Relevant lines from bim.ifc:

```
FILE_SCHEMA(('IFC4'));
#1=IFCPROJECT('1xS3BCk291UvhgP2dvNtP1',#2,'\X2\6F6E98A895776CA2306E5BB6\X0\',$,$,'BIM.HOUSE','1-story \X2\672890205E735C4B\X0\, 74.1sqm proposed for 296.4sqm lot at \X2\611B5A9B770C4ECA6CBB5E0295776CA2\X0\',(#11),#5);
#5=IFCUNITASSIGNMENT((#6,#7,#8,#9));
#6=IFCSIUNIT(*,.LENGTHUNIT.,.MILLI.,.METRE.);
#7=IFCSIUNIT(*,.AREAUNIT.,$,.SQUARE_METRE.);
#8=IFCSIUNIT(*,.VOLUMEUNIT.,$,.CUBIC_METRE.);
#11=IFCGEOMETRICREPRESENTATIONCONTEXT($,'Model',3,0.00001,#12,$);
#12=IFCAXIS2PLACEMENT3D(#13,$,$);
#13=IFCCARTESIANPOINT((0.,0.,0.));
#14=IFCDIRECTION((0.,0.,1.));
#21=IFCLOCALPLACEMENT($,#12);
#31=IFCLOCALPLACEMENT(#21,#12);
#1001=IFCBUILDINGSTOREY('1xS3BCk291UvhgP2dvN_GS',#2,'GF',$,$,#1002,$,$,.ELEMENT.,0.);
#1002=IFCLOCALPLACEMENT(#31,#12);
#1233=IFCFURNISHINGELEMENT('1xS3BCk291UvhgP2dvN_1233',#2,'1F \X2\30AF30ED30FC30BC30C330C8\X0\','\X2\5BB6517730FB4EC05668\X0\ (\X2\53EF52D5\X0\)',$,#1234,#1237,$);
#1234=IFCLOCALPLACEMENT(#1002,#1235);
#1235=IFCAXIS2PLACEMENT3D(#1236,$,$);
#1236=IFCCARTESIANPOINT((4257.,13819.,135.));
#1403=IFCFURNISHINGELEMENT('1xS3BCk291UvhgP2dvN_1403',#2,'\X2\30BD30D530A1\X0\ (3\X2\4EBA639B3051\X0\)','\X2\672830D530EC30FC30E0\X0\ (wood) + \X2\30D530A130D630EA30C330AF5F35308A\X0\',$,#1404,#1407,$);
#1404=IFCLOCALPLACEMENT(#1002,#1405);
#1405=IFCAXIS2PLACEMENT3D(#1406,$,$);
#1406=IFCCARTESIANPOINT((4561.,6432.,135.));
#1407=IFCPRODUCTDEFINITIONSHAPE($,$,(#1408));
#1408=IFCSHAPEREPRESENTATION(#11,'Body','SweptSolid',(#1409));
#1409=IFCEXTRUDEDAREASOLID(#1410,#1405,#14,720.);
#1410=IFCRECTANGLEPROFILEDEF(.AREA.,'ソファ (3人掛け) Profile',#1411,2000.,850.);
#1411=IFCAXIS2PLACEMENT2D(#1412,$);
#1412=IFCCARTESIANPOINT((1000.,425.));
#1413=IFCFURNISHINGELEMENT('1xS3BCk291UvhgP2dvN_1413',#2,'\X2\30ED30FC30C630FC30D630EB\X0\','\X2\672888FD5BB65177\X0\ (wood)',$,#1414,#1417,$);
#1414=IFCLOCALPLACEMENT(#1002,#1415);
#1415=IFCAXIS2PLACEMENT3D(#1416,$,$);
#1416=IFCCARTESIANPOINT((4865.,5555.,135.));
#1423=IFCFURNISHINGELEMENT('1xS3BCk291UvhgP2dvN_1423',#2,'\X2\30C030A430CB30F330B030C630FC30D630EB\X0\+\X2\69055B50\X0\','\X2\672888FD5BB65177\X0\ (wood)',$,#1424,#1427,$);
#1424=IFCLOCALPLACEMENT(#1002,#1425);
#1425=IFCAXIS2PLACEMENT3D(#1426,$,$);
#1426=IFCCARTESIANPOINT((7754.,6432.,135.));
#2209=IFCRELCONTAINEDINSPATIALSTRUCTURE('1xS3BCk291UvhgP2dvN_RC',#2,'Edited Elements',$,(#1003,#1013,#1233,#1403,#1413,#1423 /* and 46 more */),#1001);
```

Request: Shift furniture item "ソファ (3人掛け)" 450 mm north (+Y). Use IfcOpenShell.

```python
import ifcopenshell
import ifcopenshell.api.geometry
import ifcopenshell.util.placement
import ifcopenshell.util.unit

model = ifcopenshell.open("bim.ifc")
unit_scale = ifcopenshell.util.unit.calculate_unit_scale(model)

item = model.by_guid("1xS3BCk291UvhgP2dvN_1403")
matrix = ifcopenshell.util.placement.get_local_placement(item.ObjectPlacement)
matrix[1, 3] += 0.45 / unit_scale
ifcopenshell.api.geometry.edit_object_placement(model, product=item, matrix=matrix, is_si=False)

print(ifcopenshell.util.placement.get_local_placement(item.ObjectPlacement).round(3) + 0.0)

model.write("bim_edited.ifc")
```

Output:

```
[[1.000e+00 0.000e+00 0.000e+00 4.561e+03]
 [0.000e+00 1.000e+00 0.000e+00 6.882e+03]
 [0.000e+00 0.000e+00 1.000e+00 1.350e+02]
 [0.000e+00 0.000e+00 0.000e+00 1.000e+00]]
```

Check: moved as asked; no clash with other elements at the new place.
